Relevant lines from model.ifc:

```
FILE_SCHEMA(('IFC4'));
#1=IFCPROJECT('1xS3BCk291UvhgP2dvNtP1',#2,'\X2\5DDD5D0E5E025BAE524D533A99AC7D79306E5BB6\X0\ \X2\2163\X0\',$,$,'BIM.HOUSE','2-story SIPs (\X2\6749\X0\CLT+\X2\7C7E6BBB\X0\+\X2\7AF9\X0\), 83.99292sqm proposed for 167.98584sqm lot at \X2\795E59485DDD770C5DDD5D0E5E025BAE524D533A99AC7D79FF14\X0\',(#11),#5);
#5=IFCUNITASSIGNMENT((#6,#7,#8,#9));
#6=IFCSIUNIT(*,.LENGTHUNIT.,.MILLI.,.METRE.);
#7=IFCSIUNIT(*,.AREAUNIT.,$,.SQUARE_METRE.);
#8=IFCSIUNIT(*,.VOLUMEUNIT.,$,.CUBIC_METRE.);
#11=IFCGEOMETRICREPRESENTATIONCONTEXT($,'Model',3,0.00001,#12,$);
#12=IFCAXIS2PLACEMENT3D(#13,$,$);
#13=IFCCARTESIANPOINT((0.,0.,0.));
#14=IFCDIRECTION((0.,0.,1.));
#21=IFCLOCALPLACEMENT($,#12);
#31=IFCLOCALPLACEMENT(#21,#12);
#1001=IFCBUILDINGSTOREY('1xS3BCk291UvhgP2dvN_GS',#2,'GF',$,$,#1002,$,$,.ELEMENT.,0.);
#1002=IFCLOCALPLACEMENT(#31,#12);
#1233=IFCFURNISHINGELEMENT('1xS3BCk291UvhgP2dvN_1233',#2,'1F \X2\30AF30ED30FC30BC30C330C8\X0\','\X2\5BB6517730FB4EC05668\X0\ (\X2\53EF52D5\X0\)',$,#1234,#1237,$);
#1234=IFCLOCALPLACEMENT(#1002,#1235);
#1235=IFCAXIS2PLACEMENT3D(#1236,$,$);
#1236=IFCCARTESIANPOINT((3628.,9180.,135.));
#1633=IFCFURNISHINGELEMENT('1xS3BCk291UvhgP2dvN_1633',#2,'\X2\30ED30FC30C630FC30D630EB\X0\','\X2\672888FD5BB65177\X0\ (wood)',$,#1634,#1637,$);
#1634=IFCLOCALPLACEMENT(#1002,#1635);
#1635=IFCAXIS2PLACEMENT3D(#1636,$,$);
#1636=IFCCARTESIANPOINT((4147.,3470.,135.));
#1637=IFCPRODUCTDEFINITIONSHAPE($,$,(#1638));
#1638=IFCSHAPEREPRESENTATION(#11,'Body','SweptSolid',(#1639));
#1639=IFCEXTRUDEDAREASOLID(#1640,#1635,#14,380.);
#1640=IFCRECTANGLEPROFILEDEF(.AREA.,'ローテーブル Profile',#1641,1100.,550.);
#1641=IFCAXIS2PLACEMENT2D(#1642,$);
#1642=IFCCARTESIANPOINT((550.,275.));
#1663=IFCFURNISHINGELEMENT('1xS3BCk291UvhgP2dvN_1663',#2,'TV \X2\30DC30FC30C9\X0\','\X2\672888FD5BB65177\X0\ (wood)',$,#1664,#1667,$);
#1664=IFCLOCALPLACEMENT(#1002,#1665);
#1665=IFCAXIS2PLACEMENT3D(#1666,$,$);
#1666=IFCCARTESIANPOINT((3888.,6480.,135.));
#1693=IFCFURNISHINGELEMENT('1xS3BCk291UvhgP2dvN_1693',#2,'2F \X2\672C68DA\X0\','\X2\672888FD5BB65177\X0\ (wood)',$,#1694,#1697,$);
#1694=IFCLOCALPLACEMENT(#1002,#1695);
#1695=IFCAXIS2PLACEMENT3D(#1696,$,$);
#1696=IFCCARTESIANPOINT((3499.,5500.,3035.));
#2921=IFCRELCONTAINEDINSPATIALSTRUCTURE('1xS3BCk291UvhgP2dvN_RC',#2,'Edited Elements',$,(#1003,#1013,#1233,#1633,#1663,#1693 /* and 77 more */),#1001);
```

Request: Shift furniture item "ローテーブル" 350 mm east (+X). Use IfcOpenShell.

```python
import ifcopenshell
import ifcopenshell.api.geometry
import ifcopenshell.util.placement
import ifcopenshell.util.unit

model = ifcopenshell.open("model.ifc")
unit_scale = ifcopenshell.util.unit.calculate_unit_scale(model)

item = model.by_guid("1xS3BCk291UvhgP2dvN_1633")
matrix = ifcopenshell.util.placement.get_local_placement(item.ObjectPlacement)
matrix[0, 3] += 0.35 / unit_scale
ifcopenshell.api.geometry.edit_object_placement(model, product=item, matrix=matrix, is_si=False)

print(ifcopenshell.util.placement.get_local_placement(item.ObjectPlacement).round(3) + 0.0)

model.write("model_updated.ifc")
```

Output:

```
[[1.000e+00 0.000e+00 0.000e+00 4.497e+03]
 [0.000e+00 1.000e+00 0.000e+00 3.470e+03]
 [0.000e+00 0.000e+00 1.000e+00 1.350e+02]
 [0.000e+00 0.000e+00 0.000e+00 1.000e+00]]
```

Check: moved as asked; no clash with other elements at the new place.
